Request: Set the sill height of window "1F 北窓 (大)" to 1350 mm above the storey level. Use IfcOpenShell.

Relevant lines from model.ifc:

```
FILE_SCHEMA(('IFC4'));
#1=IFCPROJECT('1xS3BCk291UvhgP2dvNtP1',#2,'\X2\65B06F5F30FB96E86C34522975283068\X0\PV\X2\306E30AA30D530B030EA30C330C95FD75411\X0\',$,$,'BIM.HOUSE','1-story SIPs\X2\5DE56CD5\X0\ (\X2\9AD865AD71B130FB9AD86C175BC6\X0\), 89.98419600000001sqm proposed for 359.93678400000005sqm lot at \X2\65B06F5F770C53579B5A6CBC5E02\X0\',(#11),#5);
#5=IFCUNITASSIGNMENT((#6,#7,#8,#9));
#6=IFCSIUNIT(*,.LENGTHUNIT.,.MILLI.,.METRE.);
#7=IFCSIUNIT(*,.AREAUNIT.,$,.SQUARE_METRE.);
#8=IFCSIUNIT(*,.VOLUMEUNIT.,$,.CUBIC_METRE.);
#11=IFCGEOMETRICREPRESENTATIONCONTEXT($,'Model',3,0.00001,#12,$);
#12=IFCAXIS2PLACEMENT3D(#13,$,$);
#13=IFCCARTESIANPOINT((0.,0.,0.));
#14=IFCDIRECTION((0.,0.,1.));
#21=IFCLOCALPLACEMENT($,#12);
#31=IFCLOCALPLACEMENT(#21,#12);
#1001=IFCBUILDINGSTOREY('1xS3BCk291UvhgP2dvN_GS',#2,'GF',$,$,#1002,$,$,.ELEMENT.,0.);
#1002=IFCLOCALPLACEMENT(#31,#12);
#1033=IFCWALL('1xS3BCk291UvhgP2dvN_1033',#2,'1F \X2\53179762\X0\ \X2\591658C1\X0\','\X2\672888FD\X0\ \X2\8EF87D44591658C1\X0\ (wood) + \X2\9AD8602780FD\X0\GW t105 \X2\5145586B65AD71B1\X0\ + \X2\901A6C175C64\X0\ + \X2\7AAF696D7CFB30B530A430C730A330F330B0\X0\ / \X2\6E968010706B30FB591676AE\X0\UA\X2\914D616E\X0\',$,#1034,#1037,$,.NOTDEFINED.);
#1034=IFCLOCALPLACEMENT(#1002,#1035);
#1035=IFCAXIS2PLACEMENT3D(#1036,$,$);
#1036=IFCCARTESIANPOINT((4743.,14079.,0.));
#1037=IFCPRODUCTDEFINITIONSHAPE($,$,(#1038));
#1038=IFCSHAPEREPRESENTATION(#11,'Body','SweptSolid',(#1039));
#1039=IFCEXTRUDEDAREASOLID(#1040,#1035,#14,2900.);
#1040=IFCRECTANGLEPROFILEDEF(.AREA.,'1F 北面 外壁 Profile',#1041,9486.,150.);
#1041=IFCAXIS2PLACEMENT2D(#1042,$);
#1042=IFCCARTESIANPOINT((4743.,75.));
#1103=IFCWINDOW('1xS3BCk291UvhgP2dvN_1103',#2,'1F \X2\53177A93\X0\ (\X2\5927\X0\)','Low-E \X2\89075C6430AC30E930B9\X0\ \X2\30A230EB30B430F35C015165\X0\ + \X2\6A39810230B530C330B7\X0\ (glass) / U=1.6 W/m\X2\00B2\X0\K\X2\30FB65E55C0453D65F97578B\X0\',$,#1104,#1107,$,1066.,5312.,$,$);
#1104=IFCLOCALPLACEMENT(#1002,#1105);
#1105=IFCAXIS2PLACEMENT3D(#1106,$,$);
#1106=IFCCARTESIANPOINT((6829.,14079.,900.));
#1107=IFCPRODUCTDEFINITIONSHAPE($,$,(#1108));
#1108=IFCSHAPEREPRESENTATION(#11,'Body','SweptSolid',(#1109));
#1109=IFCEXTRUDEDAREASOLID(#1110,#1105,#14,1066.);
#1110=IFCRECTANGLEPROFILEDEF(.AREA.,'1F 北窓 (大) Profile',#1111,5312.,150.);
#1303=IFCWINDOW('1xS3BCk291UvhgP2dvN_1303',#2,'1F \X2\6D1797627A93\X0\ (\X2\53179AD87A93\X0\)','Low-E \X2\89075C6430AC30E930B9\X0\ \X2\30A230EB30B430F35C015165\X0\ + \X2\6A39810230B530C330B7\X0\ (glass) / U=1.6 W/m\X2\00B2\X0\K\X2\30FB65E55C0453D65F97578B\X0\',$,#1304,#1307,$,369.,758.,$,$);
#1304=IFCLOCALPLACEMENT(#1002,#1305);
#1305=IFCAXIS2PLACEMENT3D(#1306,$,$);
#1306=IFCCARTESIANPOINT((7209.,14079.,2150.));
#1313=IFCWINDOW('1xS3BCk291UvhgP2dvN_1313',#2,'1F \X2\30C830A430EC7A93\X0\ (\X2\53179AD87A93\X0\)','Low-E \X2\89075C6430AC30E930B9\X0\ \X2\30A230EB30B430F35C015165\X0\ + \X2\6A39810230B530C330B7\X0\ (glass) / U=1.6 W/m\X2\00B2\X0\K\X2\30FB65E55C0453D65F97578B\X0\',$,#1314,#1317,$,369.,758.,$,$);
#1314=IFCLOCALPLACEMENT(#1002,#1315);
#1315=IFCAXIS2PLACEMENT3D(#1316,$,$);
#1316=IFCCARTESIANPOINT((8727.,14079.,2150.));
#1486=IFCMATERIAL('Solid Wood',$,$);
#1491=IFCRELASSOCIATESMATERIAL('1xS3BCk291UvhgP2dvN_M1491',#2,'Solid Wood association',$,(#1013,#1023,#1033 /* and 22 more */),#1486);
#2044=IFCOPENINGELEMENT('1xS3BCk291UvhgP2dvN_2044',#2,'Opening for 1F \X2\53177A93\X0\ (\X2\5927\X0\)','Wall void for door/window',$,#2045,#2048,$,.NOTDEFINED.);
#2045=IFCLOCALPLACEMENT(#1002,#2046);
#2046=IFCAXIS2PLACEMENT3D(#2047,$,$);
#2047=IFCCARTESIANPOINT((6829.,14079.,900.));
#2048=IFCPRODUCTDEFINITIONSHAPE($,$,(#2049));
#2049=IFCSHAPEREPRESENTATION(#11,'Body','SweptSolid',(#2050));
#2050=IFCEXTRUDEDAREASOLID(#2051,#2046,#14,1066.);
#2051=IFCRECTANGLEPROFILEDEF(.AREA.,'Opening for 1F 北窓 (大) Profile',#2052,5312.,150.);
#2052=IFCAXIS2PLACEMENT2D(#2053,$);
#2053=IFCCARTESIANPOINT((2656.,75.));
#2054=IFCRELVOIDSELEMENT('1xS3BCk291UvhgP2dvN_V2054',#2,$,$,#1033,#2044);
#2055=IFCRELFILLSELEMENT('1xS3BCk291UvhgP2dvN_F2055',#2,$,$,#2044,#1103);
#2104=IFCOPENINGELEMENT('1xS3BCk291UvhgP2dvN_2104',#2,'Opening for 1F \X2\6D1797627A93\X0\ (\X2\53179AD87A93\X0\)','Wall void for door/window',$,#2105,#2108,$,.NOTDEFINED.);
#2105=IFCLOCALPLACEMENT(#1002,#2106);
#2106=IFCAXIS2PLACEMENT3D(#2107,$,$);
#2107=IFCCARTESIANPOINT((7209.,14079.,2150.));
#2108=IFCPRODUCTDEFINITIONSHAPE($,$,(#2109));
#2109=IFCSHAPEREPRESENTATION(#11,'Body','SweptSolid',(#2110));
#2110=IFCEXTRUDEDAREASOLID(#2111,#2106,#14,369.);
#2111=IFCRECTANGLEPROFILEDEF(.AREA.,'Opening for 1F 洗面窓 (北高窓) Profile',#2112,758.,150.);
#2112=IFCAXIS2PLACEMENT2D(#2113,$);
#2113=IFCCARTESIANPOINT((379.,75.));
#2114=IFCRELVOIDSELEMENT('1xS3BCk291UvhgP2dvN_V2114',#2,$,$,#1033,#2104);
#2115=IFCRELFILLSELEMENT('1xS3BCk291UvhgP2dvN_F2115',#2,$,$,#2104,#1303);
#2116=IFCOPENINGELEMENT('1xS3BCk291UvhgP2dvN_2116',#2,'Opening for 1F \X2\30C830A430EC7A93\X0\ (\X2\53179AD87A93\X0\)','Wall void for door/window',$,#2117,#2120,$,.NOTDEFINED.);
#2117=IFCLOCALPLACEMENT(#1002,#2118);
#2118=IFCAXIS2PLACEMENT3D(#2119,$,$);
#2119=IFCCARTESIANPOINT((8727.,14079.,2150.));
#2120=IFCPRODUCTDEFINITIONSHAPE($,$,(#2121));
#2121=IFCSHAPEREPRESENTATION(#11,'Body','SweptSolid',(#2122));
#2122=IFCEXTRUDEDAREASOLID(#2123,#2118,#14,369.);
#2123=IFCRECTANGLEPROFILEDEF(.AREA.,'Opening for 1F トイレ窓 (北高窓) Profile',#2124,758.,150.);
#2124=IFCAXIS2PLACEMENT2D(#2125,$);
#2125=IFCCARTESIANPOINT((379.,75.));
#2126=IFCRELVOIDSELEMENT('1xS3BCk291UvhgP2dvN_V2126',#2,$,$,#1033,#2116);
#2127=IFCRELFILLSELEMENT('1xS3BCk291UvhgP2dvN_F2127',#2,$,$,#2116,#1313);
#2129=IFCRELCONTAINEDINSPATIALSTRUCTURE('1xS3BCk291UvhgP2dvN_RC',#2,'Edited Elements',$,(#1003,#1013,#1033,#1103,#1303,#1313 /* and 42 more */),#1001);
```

```python
import numpy as np
import ifcopenshell
import ifcopenshell.api.geometry
import ifcopenshell.geom
import ifcopenshell.util.element
import ifcopenshell.util.placement
import ifcopenshell.util.shape
import ifcopenshell.util.unit

model = ifcopenshell.open("model.ifc")
unit_scale = ifcopenshell.util.unit.calculate_unit_scale(model)

window = model.by_guid("1xS3BCk291UvhgP2dvN_1103")
opening = window.FillsVoids[0].RelatingOpeningElement
storey = ifcopenshell.util.element.get_container(window, ifc_class="IfcBuildingStorey")
level = ifcopenshell.util.placement.get_local_placement(storey.ObjectPlacement)[2, 3]

# The opening's origin need not be at the sill, so measure its lowest point.
shape = ifcopenshell.geom.create_shape(ifcopenshell.geom.settings(), opening)
bottom = ifcopenshell.util.shape.get_shape_bottom_elevation(shape, shape.geometry) / unit_scale
dz = level + 1.35 / unit_scale - bottom

shift = np.array([0.0, 0.0, dz])
# The window is not placed relative to its opening, so move both.
for product in (opening, window):
    matrix = ifcopenshell.util.placement.get_local_placement(product.ObjectPlacement)
    matrix[:3, 3] += shift
    ifcopenshell.api.geometry.edit_object_placement(model, product=product, matrix=matrix, is_si=False)

print(f"moved by {dz * unit_scale:+.3f} m")

model.write("model-out.ifc")
```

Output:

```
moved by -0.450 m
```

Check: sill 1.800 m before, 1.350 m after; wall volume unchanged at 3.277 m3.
